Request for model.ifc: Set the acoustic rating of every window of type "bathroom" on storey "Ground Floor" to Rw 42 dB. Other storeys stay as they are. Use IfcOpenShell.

First a look at what the model holds.

```python
import ifcopenshell
import ifcopenshell.util.element

model = ifcopenshell.open("model.ifc")
print(model.schema)
storey = next(s for s in model.by_type("IfcBuildingStorey") if s.Name == "Ground Floor")
windows = [e for e in ifcopenshell.util.element.get_decomposition(storey) if e.is_a("IfcWindow")]
seen = {}
for e in windows:
    element_type = ifcopenshell.util.element.get_type(e)
    key = (element_type.Name if element_type != e and element_type else None, ifcopenshell.util.element.get_pset(e, "Pset_WindowCommon", "AcousticRating"))
    seen[key] = seen.get(key, 0) + 1
for (name, value), count in sorted(seen.items(), key=str):
    print(count, "x", name, "|", value)
```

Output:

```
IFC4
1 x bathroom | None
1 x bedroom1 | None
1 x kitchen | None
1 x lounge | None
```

```python
import ifcopenshell
import ifcopenshell.api.pset
import ifcopenshell.util.element

model = ifcopenshell.open("model.ifc")

storey = next(s for s in model.by_type("IfcBuildingStorey") if s.Name == "Ground Floor")
windows = [e for e in ifcopenshell.util.element.get_decomposition(storey) if e.is_a("IfcWindow")]

count = 0
for e in windows:
    element_type = ifcopenshell.util.element.get_type(e)
    if element_type in (None, e) or element_type.Name != "bathroom":
        continue
    # add_pset returns the element's existing set when there is one.
    pset = ifcopenshell.api.pset.add_pset(model, product=e, name="Pset_WindowCommon")
    ifcopenshell.api.pset.edit_pset(model, pset=pset, properties={"AcousticRating": "Rw 42 dB"})
    count += 1

print(count, "windows updated")

model.write("model_updated.ifc")
```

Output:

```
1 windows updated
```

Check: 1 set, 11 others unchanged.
